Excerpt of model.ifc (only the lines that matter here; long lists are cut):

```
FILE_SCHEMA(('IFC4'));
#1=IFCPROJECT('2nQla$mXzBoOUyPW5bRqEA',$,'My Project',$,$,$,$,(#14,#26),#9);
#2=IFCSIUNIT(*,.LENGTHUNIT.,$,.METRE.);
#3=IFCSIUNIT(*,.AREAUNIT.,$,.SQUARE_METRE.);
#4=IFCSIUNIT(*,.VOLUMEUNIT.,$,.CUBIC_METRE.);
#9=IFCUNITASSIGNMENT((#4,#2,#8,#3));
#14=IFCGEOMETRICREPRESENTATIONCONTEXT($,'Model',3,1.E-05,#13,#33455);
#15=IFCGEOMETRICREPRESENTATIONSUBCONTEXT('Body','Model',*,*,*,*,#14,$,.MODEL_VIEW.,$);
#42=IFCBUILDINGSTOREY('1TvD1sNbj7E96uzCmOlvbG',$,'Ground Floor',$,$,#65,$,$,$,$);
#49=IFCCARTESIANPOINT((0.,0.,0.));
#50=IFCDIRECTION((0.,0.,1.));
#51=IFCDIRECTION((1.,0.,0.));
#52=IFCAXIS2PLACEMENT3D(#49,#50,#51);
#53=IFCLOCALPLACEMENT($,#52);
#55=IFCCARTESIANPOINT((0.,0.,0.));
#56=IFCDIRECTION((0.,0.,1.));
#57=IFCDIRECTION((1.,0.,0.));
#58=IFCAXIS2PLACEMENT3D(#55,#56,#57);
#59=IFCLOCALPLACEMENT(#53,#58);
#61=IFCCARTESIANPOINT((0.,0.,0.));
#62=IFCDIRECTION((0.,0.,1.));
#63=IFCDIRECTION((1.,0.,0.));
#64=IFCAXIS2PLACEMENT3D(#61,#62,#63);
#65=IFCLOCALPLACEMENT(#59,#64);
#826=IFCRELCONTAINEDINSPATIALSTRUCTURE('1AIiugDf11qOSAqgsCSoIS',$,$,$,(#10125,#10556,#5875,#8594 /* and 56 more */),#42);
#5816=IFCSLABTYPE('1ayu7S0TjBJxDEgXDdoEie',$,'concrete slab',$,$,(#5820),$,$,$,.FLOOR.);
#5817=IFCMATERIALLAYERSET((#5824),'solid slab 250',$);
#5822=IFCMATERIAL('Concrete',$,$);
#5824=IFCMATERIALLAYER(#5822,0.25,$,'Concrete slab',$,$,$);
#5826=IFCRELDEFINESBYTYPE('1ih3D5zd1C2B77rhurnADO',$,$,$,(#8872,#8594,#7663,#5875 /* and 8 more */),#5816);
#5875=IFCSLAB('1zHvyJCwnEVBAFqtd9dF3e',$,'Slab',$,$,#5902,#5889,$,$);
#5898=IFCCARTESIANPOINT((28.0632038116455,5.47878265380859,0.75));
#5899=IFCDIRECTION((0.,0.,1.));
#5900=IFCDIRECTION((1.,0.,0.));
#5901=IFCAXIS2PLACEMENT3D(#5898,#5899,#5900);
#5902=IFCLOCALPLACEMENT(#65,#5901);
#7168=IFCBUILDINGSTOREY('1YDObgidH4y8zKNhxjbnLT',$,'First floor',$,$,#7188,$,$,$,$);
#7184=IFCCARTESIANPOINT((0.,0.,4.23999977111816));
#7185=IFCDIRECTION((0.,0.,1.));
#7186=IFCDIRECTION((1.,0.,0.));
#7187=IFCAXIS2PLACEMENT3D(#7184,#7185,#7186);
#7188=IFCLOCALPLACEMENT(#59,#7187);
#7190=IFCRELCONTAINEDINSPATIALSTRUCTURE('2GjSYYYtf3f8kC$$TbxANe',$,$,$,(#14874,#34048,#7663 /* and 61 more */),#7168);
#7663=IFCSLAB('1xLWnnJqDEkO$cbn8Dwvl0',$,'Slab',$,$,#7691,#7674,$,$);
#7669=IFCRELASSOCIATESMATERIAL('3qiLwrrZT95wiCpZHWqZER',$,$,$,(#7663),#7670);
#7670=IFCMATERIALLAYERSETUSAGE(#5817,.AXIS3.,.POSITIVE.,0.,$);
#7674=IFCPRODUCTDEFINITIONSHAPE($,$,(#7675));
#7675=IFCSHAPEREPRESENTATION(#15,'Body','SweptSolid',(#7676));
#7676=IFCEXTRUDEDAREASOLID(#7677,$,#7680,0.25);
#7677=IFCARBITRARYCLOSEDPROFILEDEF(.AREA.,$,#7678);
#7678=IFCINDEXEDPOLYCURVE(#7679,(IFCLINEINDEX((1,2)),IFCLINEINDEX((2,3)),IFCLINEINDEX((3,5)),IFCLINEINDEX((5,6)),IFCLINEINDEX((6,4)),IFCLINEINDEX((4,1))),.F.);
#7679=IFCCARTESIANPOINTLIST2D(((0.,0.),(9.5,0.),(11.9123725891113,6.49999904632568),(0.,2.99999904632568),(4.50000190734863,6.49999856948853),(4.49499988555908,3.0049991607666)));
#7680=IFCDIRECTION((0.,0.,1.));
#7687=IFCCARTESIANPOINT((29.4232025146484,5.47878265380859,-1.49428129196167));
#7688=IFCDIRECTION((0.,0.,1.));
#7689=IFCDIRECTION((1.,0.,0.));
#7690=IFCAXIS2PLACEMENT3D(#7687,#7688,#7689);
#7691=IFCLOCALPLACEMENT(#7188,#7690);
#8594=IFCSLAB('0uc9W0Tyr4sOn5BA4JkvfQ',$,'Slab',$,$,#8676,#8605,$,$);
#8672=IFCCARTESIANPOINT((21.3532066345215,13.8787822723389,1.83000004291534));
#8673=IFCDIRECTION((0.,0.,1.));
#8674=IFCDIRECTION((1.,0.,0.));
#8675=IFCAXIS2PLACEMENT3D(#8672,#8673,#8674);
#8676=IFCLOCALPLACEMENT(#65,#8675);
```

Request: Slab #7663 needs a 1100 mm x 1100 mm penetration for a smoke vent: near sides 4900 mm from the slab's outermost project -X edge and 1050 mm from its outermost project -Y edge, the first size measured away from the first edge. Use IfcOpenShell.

```python
import numpy as np
import ifcopenshell
import ifcopenshell.api.feature
import ifcopenshell.api.geometry
import ifcopenshell.api.root
import ifcopenshell.geom
import ifcopenshell.util.placement
import ifcopenshell.util.representation
import ifcopenshell.util.shape
import ifcopenshell.util.unit

model = ifcopenshell.open("model.ifc")
unit_scale = ifcopenshell.util.unit.calculate_unit_scale(model)
settings = ifcopenshell.geom.settings()


def volume(element):
    """Net volume in cubic metres, openings subtracted."""
    shape = ifcopenshell.geom.create_shape(settings, element)
    return ifcopenshell.util.shape.get_volume(shape.geometry)


slab = model.by_id(7663)
before = volume(slab)

# Extent in the slab's own axes, in metres. The edges named are its -X and -Y sides.
slab_shape = ifcopenshell.geom.create_shape(settings, slab)
vertices = ifcopenshell.util.shape.get_vertices(slab_shape.geometry)
x_min, y_min, bottom = vertices.min(axis=0)
top = vertices[:, 2].max()

opening = ifcopenshell.api.root.create_entity(model, ifc_class="IfcOpeningElement", name="Smoke vent opening", predefined_type="OPENING")
context = ifcopenshell.util.representation.get_context(model, "Model", "Body", "MODEL_VIEW")
width, depth = 1.1, 1.1
outline = [(0.0, 0.0), (width, 0.0), (width, depth), (0.0, depth), (0.0, 0.0)]
# Overshoot both faces by 50 mm so the cut is clean.
shape = ifcopenshell.api.geometry.add_slab_representation(
    model, context=context, depth=top - bottom + 0.1, polyline=outline
)
ifcopenshell.api.geometry.assign_representation(model, product=opening, representation=shape)

matrix = ifcopenshell.util.placement.get_local_placement(slab.ObjectPlacement)
matrix[:, 3] = matrix @ np.append(np.array([x_min + 4.9, y_min + 1.05, bottom - 0.05]) / unit_scale, 1.0)
ifcopenshell.api.geometry.edit_object_placement(model, product=opening, matrix=matrix, is_si=False)
ifcopenshell.api.feature.add_feature(model, feature=opening, element=slab)

after = volume(slab)

print(f"slab volume {before:.3f} -> {after:.3f} m3")

model.write("model_edited.ifc")
```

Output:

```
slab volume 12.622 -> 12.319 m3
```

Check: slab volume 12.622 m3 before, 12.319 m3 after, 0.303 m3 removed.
